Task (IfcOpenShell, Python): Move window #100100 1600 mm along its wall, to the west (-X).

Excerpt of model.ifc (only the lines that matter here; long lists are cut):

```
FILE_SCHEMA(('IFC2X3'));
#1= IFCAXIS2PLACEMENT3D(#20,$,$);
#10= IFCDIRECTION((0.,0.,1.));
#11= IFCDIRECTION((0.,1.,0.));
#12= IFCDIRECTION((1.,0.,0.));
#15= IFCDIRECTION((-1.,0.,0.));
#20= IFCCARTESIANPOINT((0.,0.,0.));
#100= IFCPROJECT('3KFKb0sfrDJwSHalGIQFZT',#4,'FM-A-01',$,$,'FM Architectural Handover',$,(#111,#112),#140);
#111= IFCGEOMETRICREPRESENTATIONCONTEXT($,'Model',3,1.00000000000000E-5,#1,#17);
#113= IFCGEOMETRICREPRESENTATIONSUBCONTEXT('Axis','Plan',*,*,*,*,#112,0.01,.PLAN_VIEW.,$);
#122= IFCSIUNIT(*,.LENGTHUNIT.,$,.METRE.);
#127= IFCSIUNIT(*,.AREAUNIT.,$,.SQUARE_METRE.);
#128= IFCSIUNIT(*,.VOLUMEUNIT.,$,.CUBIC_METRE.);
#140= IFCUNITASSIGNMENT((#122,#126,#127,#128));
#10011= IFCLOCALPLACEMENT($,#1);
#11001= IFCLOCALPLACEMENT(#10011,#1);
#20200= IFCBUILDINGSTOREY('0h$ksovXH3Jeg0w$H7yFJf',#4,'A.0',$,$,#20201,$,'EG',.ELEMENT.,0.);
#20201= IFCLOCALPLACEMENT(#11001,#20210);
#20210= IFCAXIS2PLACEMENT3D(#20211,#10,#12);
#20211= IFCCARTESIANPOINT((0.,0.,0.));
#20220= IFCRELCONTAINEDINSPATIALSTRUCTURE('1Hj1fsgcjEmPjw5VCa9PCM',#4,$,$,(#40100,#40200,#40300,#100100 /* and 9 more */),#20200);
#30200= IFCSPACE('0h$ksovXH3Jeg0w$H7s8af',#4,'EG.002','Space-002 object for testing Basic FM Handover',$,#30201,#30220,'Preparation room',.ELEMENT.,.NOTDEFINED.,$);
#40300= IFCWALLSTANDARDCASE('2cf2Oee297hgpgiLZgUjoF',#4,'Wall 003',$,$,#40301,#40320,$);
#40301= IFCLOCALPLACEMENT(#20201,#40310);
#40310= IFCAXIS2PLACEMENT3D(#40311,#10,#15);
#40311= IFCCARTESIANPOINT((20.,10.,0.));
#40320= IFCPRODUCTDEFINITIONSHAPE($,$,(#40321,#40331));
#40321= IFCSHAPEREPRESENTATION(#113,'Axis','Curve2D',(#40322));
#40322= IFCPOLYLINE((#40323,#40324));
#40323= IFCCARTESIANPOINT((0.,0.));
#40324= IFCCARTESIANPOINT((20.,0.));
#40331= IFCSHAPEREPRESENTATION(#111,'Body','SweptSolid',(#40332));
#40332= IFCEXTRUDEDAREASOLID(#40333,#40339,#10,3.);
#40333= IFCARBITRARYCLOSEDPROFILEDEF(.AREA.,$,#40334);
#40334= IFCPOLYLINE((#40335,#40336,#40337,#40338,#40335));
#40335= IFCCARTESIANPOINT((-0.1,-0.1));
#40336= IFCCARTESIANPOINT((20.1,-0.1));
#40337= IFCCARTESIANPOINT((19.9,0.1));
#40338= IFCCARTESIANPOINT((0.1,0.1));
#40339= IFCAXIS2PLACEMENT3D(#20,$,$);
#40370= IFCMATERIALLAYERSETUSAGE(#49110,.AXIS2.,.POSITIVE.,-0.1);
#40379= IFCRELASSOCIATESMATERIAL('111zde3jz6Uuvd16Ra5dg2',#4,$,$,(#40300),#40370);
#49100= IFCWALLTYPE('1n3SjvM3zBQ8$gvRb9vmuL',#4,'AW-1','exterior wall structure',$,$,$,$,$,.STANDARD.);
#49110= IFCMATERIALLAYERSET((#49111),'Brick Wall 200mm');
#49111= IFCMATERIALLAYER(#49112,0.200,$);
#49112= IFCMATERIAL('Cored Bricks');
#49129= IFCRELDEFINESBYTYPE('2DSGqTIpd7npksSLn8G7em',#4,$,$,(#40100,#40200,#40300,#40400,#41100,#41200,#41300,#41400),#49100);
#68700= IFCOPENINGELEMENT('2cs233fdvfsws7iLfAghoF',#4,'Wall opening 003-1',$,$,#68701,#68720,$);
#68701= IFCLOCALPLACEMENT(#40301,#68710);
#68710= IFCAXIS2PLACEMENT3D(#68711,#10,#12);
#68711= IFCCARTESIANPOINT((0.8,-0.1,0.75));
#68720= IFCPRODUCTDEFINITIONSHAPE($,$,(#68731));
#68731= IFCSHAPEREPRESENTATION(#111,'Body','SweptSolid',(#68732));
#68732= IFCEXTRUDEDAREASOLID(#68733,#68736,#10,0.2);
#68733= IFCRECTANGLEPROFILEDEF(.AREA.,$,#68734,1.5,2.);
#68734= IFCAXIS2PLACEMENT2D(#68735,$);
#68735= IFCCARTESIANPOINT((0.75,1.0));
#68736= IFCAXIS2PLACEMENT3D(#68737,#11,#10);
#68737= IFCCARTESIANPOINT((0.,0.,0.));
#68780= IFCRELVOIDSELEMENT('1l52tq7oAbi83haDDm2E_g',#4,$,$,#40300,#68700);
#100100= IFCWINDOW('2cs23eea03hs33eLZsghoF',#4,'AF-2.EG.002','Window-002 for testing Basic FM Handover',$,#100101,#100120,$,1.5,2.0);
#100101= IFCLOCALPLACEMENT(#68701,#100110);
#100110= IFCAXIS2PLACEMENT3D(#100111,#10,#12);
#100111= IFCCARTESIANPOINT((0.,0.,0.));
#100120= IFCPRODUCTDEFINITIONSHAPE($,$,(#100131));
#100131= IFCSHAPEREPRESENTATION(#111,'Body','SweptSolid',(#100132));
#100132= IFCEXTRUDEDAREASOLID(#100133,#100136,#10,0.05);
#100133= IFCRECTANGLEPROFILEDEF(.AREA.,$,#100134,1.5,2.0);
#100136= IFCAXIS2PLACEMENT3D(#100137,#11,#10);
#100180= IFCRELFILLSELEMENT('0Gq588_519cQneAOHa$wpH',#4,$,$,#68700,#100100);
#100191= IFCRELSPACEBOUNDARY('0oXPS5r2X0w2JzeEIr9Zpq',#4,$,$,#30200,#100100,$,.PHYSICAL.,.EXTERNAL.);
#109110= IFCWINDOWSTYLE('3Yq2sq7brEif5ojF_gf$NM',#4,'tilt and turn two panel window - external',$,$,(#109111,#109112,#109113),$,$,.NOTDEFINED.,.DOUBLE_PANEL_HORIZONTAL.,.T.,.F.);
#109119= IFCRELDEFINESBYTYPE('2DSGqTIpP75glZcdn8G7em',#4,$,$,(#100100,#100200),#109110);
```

```python
import ifcopenshell
import ifcopenshell.api.geometry
import ifcopenshell.util.placement
import ifcopenshell.util.unit

model = ifcopenshell.open("model.ifc")
unit_scale = ifcopenshell.util.unit.calculate_unit_scale(model)

window = model.by_guid("2cs23eea03hs33eLZsghoF")
opening = window.FillsVoids[0].RelatingOpeningElement
wall = opening.VoidsElements[0].RelatingBuildingElement

wall_matrix = ifcopenshell.util.placement.get_local_placement(wall.ObjectPlacement)
shift = wall_matrix[:3, 0] * 1.6 / unit_scale
before = ifcopenshell.util.placement.get_local_placement(window.ObjectPlacement)[:3, 3].copy()

# The window is placed relative to its opening, so it follows when the opening moves.
matrix = ifcopenshell.util.placement.get_local_placement(opening.ObjectPlacement)
matrix[:3, 3] += shift
ifcopenshell.api.geometry.edit_object_placement(
    model, product=opening, matrix=matrix, is_si=False, should_transform_children=True
)

after = ifcopenshell.util.placement.get_local_placement(window.ObjectPlacement)[:3, 3]
print("window moved by", (after - before).round(3) + 0.0)

model.write("model_rev.ifc")
```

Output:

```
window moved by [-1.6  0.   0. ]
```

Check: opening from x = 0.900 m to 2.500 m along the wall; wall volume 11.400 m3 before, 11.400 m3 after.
